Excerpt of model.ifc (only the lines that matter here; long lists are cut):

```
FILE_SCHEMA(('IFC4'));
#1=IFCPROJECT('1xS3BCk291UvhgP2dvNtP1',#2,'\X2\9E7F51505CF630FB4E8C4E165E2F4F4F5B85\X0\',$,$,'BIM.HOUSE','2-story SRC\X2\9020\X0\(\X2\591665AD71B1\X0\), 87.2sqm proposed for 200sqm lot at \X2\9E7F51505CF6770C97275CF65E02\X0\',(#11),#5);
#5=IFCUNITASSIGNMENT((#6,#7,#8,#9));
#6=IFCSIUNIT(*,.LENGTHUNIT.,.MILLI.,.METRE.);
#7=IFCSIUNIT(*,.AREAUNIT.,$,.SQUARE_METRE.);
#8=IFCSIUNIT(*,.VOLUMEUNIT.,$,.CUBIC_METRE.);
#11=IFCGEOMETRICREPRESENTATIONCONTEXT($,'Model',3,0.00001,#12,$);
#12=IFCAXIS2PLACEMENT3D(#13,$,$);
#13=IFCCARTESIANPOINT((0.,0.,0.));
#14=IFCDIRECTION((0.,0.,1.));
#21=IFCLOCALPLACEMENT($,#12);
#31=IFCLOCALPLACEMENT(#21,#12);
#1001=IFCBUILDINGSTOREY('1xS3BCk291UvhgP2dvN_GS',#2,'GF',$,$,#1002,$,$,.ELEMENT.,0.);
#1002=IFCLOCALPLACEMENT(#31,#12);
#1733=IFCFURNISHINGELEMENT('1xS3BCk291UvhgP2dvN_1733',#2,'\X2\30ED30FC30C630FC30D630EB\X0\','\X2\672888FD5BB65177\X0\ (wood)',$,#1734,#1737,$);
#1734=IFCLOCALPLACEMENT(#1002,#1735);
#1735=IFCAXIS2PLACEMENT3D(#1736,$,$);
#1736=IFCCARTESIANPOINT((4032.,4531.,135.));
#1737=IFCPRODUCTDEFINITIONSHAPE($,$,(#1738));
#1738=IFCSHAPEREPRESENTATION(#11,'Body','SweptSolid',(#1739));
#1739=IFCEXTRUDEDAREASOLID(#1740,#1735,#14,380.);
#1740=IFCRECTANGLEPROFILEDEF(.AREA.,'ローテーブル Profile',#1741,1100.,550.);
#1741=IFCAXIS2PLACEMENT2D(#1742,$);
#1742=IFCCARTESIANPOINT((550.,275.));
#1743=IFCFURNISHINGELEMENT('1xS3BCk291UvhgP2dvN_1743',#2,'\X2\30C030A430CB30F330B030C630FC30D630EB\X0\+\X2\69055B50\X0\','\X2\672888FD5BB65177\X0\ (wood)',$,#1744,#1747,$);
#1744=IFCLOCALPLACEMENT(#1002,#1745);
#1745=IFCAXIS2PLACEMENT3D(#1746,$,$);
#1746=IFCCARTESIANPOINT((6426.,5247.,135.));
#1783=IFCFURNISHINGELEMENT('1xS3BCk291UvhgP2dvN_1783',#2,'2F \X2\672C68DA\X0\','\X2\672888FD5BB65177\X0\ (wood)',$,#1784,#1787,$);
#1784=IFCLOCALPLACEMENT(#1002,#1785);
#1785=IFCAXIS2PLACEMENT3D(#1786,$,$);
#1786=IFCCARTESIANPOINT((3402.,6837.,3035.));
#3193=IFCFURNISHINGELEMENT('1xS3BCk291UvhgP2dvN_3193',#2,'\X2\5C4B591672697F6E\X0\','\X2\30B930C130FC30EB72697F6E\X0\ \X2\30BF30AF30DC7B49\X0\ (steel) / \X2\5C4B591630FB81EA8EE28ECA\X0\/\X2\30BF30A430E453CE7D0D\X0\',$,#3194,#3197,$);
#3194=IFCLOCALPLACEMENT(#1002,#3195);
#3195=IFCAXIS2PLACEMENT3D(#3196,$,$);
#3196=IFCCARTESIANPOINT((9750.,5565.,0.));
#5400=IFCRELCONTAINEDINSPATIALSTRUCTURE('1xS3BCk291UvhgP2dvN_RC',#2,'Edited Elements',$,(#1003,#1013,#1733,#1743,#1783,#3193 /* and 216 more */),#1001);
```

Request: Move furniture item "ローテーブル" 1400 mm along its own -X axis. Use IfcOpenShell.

```python
import ifcopenshell
import ifcopenshell.api.geometry
import ifcopenshell.util.placement

model = ifcopenshell.open("model.ifc")

item = model.by_guid("1xS3BCk291UvhgP2dvN_1733")
matrix = ifcopenshell.util.placement.get_local_placement(item.ObjectPlacement)
matrix[:3, 3] -= matrix[:3, 0] * 1400.0
ifcopenshell.api.geometry.edit_object_placement(model, product=item, matrix=matrix, is_si=False)

print(ifcopenshell.util.placement.get_local_placement(item.ObjectPlacement).round(3) + 0.0)

model.write("model_v2.ifc")
```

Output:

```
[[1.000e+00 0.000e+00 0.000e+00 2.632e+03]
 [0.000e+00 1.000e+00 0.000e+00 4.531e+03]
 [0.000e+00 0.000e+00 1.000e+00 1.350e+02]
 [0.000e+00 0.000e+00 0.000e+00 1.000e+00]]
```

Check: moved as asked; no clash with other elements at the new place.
